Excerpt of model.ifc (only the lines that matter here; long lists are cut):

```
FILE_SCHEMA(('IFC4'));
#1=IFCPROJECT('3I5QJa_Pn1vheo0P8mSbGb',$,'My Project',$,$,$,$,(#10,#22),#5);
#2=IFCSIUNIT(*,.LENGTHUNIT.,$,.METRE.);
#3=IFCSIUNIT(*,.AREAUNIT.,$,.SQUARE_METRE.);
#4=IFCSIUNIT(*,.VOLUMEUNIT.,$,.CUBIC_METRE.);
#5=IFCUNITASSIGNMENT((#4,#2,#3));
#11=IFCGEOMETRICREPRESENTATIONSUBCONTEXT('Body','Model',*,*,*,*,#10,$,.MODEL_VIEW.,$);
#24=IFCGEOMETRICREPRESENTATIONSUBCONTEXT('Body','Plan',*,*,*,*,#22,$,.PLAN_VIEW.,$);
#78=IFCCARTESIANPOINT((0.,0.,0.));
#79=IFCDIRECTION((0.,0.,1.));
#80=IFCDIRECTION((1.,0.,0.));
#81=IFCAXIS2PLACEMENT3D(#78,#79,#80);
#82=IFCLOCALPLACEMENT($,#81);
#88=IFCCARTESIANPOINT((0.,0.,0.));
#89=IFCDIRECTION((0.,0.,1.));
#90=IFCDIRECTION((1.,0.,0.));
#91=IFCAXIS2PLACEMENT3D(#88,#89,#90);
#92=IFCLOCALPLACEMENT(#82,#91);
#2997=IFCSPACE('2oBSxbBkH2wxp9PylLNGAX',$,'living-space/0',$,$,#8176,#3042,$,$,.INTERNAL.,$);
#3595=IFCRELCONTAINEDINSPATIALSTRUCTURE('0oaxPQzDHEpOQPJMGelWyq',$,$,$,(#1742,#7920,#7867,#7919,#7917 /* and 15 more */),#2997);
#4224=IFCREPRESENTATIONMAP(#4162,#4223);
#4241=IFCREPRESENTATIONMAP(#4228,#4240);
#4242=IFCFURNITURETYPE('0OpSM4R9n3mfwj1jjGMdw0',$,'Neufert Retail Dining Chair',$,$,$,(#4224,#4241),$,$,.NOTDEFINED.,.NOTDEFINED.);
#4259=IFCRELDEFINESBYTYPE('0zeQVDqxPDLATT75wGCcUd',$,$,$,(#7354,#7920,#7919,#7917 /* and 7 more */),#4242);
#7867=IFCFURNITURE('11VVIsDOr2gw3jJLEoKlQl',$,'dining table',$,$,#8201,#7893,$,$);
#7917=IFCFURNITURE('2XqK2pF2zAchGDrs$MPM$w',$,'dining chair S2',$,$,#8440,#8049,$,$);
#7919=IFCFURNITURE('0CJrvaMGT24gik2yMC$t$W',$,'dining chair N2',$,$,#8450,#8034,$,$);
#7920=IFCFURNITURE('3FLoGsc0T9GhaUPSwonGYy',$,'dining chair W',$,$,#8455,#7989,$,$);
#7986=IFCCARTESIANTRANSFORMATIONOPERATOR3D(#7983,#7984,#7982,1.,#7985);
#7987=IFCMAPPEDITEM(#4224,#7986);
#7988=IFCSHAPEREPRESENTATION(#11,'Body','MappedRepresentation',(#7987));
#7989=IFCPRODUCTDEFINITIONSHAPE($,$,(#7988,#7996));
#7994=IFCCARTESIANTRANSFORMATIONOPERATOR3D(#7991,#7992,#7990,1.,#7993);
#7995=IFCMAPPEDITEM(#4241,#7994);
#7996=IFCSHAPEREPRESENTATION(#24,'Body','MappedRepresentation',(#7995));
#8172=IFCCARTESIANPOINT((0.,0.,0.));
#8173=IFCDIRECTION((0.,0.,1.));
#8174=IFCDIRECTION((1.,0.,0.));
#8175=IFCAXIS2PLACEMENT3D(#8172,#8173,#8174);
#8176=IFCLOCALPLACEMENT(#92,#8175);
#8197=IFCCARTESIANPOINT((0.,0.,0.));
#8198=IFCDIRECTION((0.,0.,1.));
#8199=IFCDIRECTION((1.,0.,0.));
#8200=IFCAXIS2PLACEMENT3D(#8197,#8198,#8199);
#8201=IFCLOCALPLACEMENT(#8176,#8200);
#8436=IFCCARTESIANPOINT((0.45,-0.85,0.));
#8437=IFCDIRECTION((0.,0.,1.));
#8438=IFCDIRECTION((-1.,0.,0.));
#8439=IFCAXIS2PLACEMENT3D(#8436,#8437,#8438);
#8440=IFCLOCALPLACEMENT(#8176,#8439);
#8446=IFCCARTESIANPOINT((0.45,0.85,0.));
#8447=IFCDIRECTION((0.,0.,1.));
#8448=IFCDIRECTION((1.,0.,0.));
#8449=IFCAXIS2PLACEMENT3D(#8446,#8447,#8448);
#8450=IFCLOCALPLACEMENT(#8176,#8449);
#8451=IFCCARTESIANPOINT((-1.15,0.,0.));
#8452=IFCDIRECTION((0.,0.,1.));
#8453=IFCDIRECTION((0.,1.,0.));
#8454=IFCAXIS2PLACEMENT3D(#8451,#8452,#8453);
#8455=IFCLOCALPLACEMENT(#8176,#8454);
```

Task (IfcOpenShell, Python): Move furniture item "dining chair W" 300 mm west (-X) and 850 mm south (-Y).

```python
import ifcopenshell
import ifcopenshell.api.geometry
import ifcopenshell.util.placement
import ifcopenshell.util.unit

model = ifcopenshell.open("model.ifc")
unit_scale = ifcopenshell.util.unit.calculate_unit_scale(model)

item = model.by_guid("3FLoGsc0T9GhaUPSwonGYy")
matrix = ifcopenshell.util.placement.get_local_placement(item.ObjectPlacement)
matrix[0, 3] -= 0.3 / unit_scale
matrix[1, 3] -= 0.85 / unit_scale
ifcopenshell.api.geometry.edit_object_placement(model, product=item, matrix=matrix, is_si=False)

print(ifcopenshell.util.placement.get_local_placement(item.ObjectPlacement).round(3) + 0.0)

model.write("model_edited.ifc")
```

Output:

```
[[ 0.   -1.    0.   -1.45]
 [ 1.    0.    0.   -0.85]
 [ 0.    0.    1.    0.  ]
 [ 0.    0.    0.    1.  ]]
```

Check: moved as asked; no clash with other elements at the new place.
